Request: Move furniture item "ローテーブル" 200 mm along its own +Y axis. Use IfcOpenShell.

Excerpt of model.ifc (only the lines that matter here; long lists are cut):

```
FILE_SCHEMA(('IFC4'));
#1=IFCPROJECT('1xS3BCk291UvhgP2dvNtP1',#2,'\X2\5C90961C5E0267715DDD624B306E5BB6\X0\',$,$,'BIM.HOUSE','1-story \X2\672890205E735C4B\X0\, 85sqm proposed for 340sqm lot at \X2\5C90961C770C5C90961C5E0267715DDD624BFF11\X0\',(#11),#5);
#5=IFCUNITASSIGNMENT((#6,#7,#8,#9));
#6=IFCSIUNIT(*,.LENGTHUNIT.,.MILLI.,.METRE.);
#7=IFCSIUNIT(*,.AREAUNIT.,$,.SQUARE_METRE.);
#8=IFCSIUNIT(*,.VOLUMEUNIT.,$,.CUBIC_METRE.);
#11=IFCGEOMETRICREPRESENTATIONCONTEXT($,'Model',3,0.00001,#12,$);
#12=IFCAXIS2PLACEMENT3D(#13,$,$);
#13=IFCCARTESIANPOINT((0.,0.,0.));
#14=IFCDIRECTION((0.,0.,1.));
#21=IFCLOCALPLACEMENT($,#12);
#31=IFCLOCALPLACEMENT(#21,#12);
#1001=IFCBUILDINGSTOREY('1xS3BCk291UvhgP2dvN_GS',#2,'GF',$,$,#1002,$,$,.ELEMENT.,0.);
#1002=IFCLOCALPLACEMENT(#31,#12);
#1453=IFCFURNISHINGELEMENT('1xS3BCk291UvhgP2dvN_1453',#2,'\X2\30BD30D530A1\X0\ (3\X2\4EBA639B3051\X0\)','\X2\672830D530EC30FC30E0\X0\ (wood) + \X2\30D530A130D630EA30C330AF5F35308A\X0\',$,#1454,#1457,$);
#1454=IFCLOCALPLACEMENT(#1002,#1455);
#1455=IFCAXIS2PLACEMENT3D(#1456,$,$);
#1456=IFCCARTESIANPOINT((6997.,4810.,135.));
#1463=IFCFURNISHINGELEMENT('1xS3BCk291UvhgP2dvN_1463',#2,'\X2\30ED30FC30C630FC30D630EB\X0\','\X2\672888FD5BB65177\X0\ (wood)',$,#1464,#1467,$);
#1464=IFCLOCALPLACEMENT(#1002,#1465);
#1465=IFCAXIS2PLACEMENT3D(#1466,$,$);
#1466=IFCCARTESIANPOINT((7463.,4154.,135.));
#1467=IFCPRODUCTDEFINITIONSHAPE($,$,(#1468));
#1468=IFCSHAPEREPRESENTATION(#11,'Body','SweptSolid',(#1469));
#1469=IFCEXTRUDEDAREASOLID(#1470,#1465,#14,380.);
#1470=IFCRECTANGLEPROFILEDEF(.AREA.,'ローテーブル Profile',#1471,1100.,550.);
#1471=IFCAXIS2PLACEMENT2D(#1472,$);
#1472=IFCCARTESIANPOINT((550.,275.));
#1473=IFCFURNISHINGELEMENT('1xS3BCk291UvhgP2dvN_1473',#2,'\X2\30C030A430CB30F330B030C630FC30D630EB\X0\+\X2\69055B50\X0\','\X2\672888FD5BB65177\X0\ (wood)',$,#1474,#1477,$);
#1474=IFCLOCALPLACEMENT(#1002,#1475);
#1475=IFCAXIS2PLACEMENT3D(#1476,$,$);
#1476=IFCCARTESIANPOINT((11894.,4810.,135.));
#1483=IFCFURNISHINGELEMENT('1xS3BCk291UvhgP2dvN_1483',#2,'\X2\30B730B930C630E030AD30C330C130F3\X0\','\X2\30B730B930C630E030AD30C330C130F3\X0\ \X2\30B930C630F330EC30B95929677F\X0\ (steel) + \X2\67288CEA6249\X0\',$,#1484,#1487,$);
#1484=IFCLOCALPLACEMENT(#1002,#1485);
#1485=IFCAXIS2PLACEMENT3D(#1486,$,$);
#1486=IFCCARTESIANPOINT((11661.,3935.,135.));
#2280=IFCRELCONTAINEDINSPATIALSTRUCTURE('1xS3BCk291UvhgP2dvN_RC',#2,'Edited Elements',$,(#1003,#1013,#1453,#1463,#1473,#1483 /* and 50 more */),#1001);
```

```python
import ifcopenshell
import ifcopenshell.api.geometry
import ifcopenshell.util.placement
import ifcopenshell.util.unit

model = ifcopenshell.open("model.ifc")
unit_scale = ifcopenshell.util.unit.calculate_unit_scale(model)

item = model.by_guid("1xS3BCk291UvhgP2dvN_1463")
matrix = ifcopenshell.util.placement.get_local_placement(item.ObjectPlacement)
matrix[:3, 3] += matrix[:3, 1] * 0.2 / unit_scale
ifcopenshell.api.geometry.edit_object_placement(model, product=item, matrix=matrix, is_si=False)

print(ifcopenshell.util.placement.get_local_placement(item.ObjectPlacement).round(3) + 0.0)

model.write("model_v2.ifc")
```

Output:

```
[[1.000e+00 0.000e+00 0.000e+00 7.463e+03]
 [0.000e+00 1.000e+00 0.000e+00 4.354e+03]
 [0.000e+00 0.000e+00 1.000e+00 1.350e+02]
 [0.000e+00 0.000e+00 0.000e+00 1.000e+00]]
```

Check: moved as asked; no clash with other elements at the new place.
